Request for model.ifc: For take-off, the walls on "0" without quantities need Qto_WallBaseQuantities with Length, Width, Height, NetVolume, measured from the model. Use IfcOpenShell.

First a look at what the model holds.

```python
import ifcopenshell
import ifcopenshell.util.element
import ifcopenshell.util.unit

model = ifcopenshell.open("model.ifc")
print(model.schema)
for unit_type in ("LENGTHUNIT", "AREAUNIT", "VOLUMEUNIT"):
    print(unit_type, ifcopenshell.util.unit.calculate_unit_scale(model, unit_type))
storey = next(s for s in model.by_type("IfcBuildingStorey") if s.Name == "0")
walls = [e for e in ifcopenshell.util.element.get_decomposition(storey) if e.is_a("IfcWall")]
for e in sorted(walls, key=lambda e: e.id()):
    print(e.id(), e.is_a(), e.Name, list(ifcopenshell.util.element.get_psets(e, qtos_only=True)), sep=" | ")
```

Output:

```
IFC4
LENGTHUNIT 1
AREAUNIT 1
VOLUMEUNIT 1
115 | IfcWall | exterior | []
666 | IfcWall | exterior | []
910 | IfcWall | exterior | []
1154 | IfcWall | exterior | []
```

```python
import ifcopenshell
import ifcopenshell.api.pset
import ifcopenshell.geom
import ifcopenshell.util.element
import ifcopenshell.util.shape
import ifcopenshell.util.unit

model = ifcopenshell.open("model.ifc")
unit_scale = ifcopenshell.util.unit.calculate_unit_scale(model)
volume_scale = ifcopenshell.util.unit.calculate_unit_scale(model, "VOLUMEUNIT")
settings = ifcopenshell.geom.settings()

storey = next(s for s in model.by_type("IfcBuildingStorey") if s.Name == "0")
walls = [e for e in ifcopenshell.util.element.get_decomposition(storey) if e.is_a("IfcWall")]

for e in sorted(walls, key=lambda e: e.id()):
    if ifcopenshell.util.element.get_psets(e, qtos_only=True, should_inherit=False):
        continue
    # Geometry comes back in metres, in the element's own axes.
    shape = ifcopenshell.geom.create_shape(settings, e)
    values = {
        "Length": ifcopenshell.util.shape.get_x(shape.geometry) / unit_scale,
        "Width": ifcopenshell.util.shape.get_y(shape.geometry) / unit_scale,
        "Height": ifcopenshell.util.shape.get_z(shape.geometry) / unit_scale,
        "NetVolume": ifcopenshell.util.shape.get_volume(shape.geometry) / volume_scale,
    }
    qto = ifcopenshell.api.pset.add_qto(model, product=e, name="Qto_WallBaseQuantities")
    ifcopenshell.api.pset.edit_qto(model, qto=qto, properties=values)
    print(e.id(), {k: round(v, 3) for k, v in values.items()})

model.write("model_updated.ifc")
```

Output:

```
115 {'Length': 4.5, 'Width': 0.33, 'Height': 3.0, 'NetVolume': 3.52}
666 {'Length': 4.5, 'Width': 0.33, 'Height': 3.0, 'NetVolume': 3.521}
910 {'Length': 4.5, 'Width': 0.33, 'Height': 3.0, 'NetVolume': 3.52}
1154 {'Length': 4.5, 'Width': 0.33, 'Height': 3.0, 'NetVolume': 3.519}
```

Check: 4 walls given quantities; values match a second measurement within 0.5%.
